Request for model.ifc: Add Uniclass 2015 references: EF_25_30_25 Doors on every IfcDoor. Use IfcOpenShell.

First a look at what the model holds.

```python
import ifcopenshell

model = ifcopenshell.open("model.ifc")
print(model.schema)
print("classifications:", [c.Name for c in model.by_type("IfcClassification")])
for ifc_class in ("IfcDoor", "IfcRoof", "IfcStair", "IfcWall", "IfcWindow"):
    print(ifc_class, len(model.by_type(ifc_class)))
```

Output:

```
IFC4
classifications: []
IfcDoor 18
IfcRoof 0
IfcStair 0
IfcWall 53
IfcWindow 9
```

```python
import ifcopenshell
import ifcopenshell.api.classification

model = ifcopenshell.open("model.ifc")

system = ifcopenshell.api.classification.add_classification(model, classification="Uniclass 2015")

codes = {
    "IfcDoor": ("EF_25_30_25", "Doors"),
}
for ifc_class, (code, name) in codes.items():
    products = model.by_type(ifc_class)
    ifcopenshell.api.classification.add_reference(
        model, products=products, classification=system, identification=code, name=name
    )
    print(code, len(products))

model.write("model_rev.ifc")
```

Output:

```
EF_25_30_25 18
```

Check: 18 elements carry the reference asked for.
